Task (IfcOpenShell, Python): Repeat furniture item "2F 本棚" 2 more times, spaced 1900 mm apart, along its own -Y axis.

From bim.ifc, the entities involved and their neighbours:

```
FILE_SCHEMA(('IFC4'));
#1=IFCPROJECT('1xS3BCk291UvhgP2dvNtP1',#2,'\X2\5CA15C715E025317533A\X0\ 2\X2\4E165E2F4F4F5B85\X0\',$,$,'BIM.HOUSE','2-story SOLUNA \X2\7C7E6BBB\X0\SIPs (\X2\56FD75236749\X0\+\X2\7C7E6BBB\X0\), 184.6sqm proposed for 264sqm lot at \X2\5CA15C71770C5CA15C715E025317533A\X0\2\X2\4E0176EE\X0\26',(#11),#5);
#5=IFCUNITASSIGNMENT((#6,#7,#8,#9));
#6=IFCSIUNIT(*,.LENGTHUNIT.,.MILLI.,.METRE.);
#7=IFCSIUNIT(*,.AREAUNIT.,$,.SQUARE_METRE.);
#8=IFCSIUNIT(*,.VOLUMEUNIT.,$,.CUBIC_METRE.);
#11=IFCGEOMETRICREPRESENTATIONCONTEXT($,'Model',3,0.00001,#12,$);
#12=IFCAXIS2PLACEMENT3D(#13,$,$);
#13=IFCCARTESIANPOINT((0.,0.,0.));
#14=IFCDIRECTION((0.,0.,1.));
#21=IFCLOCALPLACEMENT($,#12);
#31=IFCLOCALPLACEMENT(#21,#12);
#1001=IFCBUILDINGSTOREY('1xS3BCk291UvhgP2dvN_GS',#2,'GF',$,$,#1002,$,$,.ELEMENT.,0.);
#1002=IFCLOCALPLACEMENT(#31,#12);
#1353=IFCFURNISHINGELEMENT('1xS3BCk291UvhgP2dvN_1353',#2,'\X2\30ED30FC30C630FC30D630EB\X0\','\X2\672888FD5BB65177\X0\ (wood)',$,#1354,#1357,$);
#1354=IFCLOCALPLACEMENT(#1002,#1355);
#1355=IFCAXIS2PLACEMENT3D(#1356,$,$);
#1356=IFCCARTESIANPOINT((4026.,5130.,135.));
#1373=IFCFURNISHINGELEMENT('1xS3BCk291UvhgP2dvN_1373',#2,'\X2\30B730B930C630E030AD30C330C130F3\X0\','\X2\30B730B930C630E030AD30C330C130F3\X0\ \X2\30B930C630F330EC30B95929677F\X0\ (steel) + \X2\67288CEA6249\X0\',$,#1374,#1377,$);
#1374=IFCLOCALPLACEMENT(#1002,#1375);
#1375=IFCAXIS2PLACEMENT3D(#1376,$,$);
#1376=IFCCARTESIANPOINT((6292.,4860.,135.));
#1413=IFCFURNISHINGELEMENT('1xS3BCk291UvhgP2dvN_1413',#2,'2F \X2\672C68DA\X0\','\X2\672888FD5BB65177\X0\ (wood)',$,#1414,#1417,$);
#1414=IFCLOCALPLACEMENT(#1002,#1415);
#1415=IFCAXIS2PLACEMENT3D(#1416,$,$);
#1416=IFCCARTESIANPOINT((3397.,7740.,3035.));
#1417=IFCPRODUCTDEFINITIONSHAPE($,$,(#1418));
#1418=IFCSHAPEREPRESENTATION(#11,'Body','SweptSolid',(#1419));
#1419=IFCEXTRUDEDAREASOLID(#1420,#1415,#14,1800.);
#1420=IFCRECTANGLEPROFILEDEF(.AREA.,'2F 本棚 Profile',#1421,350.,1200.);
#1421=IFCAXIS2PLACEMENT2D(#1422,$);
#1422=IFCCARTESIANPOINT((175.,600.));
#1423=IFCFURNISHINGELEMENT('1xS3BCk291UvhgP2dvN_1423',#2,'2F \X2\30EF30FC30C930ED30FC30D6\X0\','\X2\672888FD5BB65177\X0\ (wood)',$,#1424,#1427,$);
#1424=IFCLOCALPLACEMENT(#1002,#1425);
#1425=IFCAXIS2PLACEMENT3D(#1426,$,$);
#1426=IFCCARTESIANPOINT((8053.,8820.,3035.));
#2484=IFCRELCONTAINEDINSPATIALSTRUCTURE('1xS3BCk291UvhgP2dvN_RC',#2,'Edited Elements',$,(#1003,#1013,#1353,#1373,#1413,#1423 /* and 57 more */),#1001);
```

```python
import ifcopenshell
import ifcopenshell.api.geometry
import ifcopenshell.api.root
import ifcopenshell.util.element
import ifcopenshell.util.placement

model = ifcopenshell.open("bim.ifc")


def reuse_history(source, copy):
    """copy_class also copies each property set's owner history, people and application; keep the originals."""
    for rel in copy.IsDefinedBy:
        if rel.is_a("IfcRelDefinesByProperties") and (history := rel.RelatingPropertyDefinition.OwnerHistory):
            rel.RelatingPropertyDefinition.OwnerHistory = source.OwnerHistory
            ifcopenshell.util.element.remove_deep2(model, history)


source = model.by_guid("1xS3BCk291UvhgP2dvN_1413")
base = ifcopenshell.util.placement.get_local_placement(source.ObjectPlacement)
step = -base[:3, 1] * 1900.0

for i in range(1, 3):
    copy = ifcopenshell.api.root.copy_class(model, product=source)
    copy.Representation = ifcopenshell.util.element.copy_deep(
        model, source.Representation, exclude=["IfcGeometricRepresentationContext", "IfcRepresentationMap"]
    )
    reuse_history(source, copy)
    matrix = base.copy()
    matrix[:3, 3] += i * step
    print("added at", matrix[:3, 3].round(3) + 0.0)
    ifcopenshell.api.geometry.edit_object_placement(model, product=copy, matrix=matrix, is_si=False)

model.write("bim_rev.ifc")
```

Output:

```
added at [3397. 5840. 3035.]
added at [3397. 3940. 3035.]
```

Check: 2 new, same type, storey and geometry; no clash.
